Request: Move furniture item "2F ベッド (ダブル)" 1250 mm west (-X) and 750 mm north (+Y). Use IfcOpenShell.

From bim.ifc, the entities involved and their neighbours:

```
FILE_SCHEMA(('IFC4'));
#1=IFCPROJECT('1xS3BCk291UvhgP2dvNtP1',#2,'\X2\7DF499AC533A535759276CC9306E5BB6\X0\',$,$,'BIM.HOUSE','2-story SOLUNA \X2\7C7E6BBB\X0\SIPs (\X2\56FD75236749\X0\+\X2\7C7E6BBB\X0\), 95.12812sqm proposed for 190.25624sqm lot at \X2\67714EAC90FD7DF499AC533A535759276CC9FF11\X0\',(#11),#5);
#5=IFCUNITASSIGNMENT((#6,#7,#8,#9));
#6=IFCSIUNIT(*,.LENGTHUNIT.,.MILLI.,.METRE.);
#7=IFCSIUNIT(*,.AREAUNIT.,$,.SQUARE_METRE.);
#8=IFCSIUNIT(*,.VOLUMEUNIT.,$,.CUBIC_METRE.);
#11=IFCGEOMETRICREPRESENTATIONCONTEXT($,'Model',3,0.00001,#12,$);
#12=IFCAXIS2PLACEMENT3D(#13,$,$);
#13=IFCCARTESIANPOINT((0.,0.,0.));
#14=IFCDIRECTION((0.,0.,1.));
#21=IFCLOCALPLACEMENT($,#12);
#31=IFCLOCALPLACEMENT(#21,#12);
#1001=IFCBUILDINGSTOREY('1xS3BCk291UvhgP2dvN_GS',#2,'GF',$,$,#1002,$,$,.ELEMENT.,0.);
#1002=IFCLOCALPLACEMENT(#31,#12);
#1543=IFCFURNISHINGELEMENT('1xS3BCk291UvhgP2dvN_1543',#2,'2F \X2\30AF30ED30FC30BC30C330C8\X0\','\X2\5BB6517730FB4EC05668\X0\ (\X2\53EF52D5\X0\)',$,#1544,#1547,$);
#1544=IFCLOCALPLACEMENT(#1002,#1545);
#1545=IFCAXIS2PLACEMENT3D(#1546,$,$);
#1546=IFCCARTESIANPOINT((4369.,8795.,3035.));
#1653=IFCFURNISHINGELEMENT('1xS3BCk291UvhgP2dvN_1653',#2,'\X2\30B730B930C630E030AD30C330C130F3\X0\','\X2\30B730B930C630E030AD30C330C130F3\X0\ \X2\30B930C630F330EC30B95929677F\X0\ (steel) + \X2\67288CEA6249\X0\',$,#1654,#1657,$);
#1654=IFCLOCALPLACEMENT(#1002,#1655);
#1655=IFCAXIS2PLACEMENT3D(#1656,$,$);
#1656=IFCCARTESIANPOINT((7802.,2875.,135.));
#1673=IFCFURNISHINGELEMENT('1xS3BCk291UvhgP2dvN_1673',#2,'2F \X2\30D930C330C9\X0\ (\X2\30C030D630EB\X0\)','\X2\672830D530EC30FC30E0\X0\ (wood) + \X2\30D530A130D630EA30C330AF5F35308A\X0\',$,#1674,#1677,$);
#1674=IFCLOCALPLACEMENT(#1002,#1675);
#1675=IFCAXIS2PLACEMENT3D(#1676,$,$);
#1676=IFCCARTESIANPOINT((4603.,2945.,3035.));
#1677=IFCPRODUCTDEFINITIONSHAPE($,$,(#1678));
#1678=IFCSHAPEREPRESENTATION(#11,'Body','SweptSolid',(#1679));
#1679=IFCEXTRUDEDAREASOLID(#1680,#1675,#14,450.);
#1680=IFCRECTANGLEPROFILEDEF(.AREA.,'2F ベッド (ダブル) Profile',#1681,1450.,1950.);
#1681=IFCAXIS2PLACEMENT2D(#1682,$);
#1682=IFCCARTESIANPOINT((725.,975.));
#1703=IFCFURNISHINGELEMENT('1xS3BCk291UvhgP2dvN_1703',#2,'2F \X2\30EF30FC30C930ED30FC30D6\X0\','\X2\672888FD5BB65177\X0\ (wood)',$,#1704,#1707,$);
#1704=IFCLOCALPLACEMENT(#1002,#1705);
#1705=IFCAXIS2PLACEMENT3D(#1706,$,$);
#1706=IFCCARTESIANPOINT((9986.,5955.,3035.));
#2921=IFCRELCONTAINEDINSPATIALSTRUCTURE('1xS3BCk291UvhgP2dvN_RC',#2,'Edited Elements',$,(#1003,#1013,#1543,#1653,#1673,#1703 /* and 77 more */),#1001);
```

```python
import ifcopenshell
import ifcopenshell.api.geometry
import ifcopenshell.util.placement
import ifcopenshell.util.unit

model = ifcopenshell.open("bim.ifc")
unit_scale = ifcopenshell.util.unit.calculate_unit_scale(model)

item = model.by_guid("1xS3BCk291UvhgP2dvN_1673")
matrix = ifcopenshell.util.placement.get_local_placement(item.ObjectPlacement)
matrix[0, 3] -= 1.25 / unit_scale
matrix[1, 3] += 0.75 / unit_scale
ifcopenshell.api.geometry.edit_object_placement(model, product=item, matrix=matrix, is_si=False)

print(ifcopenshell.util.placement.get_local_placement(item.ObjectPlacement).round(3) + 0.0)

model.write("bim_updated.ifc")
```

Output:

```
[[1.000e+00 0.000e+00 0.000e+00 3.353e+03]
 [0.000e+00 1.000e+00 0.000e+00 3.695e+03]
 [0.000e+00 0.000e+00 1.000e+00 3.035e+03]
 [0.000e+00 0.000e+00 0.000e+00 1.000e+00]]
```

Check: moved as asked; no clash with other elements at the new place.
